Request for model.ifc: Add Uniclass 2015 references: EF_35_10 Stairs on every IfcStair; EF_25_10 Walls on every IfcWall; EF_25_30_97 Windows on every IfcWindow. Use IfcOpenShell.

First a look at what the model holds.

```python
import ifcopenshell

model = ifcopenshell.open("model.ifc")
print(model.schema)
print("classifications:", [c.Name for c in model.by_type("IfcClassification")])
for ifc_class in ("IfcDoor", "IfcRoof", "IfcStair", "IfcWall", "IfcWindow"):
    print(ifc_class, len(model.by_type(ifc_class)))
```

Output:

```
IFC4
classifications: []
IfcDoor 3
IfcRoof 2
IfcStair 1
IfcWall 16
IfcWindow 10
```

```python
import ifcopenshell
import ifcopenshell.api.classification

model = ifcopenshell.open("model.ifc")

system = ifcopenshell.api.classification.add_classification(model, classification="Uniclass 2015")

codes = {
    "IfcStair": ("EF_35_10", "Stairs"),
    "IfcWall": ("EF_25_10", "Walls"),
    "IfcWindow": ("EF_25_30_97", "Windows"),
}
for ifc_class, (code, name) in codes.items():
    products = model.by_type(ifc_class)
    ifcopenshell.api.classification.add_reference(
        model, products=products, classification=system, identification=code, name=name
    )
    print(code, len(products))

model.write("model-out.ifc")
```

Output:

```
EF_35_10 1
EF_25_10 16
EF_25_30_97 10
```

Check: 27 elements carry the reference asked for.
